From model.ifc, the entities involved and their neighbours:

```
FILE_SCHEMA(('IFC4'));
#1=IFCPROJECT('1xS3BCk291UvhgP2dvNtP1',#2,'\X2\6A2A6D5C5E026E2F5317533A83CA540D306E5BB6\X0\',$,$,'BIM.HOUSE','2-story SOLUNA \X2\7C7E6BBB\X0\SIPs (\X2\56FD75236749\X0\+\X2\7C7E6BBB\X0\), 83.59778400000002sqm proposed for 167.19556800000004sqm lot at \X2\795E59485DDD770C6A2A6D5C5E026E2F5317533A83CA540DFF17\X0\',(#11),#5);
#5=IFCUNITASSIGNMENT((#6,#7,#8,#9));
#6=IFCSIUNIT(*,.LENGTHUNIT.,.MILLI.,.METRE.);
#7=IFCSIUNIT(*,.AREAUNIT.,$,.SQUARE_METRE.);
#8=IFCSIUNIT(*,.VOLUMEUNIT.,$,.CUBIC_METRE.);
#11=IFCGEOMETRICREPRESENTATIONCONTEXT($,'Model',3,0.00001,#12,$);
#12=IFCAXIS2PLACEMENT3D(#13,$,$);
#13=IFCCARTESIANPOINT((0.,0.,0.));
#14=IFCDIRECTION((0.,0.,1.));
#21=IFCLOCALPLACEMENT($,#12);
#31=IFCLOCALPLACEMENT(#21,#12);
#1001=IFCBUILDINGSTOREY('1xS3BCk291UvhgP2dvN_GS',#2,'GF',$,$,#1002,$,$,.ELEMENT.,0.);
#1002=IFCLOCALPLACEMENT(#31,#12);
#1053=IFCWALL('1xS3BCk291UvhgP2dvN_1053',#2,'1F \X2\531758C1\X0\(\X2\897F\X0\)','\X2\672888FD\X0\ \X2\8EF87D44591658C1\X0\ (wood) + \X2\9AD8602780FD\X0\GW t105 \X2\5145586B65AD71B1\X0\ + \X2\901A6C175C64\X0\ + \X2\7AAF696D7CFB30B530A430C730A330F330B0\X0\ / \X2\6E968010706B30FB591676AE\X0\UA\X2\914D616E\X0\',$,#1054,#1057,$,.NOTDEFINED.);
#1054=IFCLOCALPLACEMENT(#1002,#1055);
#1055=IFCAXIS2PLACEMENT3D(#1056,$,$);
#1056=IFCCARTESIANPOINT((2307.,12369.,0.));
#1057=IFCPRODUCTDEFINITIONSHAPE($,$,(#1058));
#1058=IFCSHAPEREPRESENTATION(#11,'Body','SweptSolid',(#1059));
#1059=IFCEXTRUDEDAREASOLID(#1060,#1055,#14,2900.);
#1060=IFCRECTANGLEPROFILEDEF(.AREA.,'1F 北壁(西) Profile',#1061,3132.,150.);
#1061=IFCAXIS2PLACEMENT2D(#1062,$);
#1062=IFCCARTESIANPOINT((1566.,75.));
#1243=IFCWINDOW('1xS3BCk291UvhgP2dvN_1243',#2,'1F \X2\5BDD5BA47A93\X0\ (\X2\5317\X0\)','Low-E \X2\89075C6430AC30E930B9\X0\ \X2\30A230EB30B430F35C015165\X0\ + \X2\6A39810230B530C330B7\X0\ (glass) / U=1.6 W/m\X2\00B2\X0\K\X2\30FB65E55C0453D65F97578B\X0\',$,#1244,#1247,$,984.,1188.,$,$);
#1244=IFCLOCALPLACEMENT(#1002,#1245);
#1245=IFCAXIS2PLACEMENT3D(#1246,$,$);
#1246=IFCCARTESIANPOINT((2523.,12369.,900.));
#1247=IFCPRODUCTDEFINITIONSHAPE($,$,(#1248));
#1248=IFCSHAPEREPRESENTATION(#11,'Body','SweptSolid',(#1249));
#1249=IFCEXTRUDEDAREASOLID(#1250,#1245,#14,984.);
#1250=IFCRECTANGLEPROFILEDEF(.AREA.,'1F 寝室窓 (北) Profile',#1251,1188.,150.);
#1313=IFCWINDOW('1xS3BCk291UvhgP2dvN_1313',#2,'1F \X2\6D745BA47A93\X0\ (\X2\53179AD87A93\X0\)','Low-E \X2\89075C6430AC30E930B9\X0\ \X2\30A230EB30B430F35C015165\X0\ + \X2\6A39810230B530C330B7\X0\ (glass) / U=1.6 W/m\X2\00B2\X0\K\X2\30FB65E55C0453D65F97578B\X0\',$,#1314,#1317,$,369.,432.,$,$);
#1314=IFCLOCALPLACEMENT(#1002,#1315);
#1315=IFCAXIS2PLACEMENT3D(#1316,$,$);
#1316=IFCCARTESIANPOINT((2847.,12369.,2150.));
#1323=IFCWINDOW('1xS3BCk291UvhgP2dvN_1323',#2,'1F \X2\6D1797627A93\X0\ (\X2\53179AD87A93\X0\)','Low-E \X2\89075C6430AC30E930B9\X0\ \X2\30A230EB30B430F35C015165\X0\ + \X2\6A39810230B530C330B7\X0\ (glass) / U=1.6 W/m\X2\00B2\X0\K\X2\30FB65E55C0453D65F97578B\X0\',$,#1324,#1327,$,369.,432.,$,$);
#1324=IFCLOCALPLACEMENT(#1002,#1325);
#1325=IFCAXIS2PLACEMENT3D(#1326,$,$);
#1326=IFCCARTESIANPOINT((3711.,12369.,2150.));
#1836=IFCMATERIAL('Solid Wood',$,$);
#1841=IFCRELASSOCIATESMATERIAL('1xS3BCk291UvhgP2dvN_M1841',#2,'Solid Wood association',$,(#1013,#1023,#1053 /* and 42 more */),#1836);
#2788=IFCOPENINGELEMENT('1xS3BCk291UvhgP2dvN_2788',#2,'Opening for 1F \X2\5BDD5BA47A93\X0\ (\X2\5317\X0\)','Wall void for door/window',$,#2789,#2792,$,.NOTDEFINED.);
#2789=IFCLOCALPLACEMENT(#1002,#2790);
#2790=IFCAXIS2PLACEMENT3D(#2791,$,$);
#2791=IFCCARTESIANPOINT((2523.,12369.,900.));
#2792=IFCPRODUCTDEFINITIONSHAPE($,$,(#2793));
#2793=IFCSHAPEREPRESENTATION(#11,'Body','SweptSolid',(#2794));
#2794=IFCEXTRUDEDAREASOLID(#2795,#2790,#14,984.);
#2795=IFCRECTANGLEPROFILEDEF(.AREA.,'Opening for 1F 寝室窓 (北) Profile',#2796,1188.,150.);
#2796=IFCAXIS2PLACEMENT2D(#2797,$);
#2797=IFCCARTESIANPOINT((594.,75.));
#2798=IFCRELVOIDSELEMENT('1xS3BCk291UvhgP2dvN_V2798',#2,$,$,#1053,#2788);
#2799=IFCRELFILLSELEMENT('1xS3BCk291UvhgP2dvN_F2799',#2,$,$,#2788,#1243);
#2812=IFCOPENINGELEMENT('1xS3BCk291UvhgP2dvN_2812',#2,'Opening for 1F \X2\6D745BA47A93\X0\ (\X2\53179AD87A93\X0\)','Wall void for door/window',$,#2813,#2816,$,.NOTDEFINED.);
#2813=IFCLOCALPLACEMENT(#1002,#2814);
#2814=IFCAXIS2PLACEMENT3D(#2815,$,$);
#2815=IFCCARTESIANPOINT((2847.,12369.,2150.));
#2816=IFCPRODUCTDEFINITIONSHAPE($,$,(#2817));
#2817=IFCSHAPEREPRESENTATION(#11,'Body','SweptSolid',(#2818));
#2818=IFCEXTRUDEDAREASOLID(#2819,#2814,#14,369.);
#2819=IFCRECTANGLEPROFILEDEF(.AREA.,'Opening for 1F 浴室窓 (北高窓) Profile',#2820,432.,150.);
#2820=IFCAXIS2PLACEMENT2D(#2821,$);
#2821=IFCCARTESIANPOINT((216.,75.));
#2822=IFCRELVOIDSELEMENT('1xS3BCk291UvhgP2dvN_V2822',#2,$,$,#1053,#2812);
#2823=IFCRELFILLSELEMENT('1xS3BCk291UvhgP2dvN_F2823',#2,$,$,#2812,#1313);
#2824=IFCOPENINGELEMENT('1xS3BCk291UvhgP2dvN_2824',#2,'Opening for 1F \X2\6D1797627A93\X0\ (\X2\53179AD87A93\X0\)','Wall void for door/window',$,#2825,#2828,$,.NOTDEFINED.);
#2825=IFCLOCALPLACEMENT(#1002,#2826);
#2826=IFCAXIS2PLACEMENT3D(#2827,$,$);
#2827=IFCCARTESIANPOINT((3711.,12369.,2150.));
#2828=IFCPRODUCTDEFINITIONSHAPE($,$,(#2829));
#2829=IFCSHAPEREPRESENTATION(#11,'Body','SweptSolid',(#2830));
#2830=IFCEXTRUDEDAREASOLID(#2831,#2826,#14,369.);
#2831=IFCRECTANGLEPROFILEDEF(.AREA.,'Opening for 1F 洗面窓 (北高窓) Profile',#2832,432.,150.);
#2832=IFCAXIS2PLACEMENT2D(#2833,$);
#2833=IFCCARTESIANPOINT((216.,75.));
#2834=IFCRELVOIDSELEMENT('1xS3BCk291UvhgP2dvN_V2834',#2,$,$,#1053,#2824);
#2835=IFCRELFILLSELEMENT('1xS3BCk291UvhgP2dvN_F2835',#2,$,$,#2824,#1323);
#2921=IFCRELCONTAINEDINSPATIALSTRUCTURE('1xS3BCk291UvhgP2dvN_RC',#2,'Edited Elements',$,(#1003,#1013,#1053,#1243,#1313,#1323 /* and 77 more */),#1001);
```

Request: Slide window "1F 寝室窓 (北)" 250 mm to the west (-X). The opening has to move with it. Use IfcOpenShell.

```python
import ifcopenshell
import ifcopenshell.api.geometry
import ifcopenshell.util.placement
import ifcopenshell.util.unit

model = ifcopenshell.open("model.ifc")
unit_scale = ifcopenshell.util.unit.calculate_unit_scale(model)

window = model.by_guid("1xS3BCk291UvhgP2dvN_1243")
opening = window.FillsVoids[0].RelatingOpeningElement
wall = opening.VoidsElements[0].RelatingBuildingElement

wall_matrix = ifcopenshell.util.placement.get_local_placement(wall.ObjectPlacement)
shift = wall_matrix[:3, 0] * -0.25 / unit_scale
before = ifcopenshell.util.placement.get_local_placement(window.ObjectPlacement)[:3, 3].copy()

# The window is not placed relative to its opening, so move both.
for product in (opening, window):
    matrix = ifcopenshell.util.placement.get_local_placement(product.ObjectPlacement)
    matrix[:3, 3] += shift
    ifcopenshell.api.geometry.edit_object_placement(model, product=product, matrix=matrix, is_si=False)

after = ifcopenshell.util.placement.get_local_placement(window.ObjectPlacement)[:3, 3]
print("window moved by", (after - before).round(3) + 0.0)

model.write("model_rev.ifc")
```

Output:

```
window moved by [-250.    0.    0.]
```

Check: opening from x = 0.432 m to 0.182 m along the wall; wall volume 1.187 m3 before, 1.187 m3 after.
